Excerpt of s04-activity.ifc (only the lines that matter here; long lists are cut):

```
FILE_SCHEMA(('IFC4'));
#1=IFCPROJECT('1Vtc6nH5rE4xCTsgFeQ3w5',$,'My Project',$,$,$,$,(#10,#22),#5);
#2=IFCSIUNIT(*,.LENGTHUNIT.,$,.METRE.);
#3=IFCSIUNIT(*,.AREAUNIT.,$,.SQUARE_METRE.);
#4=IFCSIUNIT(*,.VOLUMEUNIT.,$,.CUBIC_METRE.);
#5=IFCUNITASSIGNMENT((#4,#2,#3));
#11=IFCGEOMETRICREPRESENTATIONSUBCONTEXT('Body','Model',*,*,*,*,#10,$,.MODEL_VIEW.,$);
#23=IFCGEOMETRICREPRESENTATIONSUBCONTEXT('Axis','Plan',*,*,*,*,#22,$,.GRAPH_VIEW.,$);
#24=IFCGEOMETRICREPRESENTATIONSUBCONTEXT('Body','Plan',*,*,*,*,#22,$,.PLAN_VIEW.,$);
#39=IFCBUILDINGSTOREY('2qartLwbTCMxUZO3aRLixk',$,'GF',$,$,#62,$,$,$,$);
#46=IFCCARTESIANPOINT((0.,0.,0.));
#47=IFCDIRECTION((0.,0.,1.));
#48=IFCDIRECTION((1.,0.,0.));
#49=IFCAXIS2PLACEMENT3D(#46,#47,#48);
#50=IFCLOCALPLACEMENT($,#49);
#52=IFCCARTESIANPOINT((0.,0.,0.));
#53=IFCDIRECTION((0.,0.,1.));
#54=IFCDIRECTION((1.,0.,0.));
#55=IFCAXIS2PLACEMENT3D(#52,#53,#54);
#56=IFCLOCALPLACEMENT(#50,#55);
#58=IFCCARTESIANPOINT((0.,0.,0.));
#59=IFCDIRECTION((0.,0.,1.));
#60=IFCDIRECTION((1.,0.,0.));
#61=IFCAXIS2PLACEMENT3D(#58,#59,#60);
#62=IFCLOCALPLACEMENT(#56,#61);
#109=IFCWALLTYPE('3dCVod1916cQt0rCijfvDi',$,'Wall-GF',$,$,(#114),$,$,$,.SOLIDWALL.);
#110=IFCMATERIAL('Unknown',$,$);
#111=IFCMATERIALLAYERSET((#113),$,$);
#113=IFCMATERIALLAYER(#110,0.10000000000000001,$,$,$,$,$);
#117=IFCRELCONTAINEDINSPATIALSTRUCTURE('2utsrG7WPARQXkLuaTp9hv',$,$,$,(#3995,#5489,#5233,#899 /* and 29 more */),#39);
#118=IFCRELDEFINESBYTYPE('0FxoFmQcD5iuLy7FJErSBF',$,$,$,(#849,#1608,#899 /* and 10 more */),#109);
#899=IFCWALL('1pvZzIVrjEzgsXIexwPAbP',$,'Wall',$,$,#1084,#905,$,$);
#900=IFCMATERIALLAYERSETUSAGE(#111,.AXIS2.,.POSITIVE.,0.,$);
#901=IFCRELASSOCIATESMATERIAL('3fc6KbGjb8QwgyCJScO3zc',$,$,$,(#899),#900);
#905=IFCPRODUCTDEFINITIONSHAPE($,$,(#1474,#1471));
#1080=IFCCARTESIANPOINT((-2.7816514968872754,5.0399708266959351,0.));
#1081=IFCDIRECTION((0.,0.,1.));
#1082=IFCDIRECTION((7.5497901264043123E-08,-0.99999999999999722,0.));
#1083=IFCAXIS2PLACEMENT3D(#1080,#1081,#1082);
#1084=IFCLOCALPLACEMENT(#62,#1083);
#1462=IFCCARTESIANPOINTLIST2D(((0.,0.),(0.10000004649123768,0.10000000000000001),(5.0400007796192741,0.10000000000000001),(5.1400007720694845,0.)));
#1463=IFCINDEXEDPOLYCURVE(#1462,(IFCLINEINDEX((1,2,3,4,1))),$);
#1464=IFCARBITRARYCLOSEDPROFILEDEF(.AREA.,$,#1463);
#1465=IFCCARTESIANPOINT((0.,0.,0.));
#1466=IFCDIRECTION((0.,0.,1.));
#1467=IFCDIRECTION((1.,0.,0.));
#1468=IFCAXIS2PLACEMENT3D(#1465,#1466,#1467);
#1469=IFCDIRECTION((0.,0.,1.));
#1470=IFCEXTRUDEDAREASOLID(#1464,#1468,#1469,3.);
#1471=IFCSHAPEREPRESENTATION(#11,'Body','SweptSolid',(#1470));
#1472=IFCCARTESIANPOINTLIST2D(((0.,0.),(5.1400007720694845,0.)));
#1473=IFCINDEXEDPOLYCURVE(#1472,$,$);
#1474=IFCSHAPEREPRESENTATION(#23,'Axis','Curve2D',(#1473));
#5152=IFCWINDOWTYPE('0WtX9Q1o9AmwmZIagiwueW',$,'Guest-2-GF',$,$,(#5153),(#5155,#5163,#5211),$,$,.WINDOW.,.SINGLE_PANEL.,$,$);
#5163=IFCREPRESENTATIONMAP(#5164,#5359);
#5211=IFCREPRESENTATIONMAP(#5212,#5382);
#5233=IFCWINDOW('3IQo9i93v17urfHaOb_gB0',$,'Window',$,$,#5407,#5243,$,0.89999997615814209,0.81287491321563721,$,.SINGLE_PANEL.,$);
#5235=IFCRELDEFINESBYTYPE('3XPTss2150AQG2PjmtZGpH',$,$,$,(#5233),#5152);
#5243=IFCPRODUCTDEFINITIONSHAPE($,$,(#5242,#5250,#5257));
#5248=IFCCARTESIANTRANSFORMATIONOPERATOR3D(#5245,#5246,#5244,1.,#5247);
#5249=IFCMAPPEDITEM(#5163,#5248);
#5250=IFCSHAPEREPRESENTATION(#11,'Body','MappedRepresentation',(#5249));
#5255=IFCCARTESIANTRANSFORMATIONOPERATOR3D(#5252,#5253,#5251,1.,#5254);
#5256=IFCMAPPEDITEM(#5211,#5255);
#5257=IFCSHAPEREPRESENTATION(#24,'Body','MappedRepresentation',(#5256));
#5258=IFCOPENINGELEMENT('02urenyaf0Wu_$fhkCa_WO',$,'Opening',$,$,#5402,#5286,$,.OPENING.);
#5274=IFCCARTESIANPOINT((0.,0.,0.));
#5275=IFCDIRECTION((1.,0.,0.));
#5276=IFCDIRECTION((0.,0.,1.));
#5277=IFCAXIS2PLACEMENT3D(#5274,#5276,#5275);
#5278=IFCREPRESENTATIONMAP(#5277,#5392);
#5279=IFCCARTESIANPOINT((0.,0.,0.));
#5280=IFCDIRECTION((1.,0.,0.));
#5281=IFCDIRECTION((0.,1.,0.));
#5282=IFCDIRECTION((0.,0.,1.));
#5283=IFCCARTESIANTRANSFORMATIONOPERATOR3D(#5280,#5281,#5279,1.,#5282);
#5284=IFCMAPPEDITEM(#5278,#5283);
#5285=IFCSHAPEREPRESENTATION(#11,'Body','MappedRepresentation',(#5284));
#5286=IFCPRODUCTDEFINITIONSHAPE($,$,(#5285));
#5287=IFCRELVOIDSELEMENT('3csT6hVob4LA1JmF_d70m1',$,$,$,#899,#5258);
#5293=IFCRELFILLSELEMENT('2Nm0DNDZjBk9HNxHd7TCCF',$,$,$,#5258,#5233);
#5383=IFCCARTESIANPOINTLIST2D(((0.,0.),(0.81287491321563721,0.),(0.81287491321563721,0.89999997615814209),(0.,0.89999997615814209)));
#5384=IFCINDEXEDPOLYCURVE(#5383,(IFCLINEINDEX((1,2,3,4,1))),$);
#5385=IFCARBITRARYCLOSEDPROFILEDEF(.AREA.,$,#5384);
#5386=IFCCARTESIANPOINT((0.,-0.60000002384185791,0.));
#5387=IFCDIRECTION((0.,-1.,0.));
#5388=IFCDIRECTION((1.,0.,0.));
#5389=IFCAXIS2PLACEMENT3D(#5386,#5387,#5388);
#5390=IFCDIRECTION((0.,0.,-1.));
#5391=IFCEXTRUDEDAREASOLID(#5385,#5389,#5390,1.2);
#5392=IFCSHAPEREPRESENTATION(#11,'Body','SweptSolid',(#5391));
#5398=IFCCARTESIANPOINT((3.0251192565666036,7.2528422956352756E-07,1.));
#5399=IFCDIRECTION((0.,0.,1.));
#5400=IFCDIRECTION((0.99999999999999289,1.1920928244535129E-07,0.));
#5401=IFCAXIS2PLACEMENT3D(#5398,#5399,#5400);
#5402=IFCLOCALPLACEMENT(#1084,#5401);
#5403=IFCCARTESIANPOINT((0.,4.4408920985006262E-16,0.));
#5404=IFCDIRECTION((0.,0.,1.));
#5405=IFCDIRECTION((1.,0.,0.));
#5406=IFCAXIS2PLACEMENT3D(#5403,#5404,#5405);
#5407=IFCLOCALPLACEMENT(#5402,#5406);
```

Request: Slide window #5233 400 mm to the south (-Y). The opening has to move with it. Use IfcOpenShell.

```python
import ifcopenshell
import ifcopenshell.api.geometry
import ifcopenshell.util.placement

model = ifcopenshell.open("s04-activity.ifc")

window = model.by_guid("3IQo9i93v17urfHaOb_gB0")
opening = window.FillsVoids[0].RelatingOpeningElement
wall = opening.VoidsElements[0].RelatingBuildingElement

wall_matrix = ifcopenshell.util.placement.get_local_placement(wall.ObjectPlacement)
shift = wall_matrix[:3, 0] * 0.4
before = ifcopenshell.util.placement.get_local_placement(window.ObjectPlacement)[:3, 3].copy()

# The window is placed relative to its opening, so it follows when the opening moves.
matrix = ifcopenshell.util.placement.get_local_placement(opening.ObjectPlacement)
matrix[:3, 3] += shift
ifcopenshell.api.geometry.edit_object_placement(
    model, product=opening, matrix=matrix, is_si=False, should_transform_children=True
)

after = ifcopenshell.util.placement.get_local_placement(window.ObjectPlacement)[:3, 3]
print("window moved by", (after - before).round(3) + 0.0)

model.write("s04-activity-out.ifc")
```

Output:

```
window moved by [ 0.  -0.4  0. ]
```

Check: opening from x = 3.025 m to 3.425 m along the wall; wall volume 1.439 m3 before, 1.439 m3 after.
